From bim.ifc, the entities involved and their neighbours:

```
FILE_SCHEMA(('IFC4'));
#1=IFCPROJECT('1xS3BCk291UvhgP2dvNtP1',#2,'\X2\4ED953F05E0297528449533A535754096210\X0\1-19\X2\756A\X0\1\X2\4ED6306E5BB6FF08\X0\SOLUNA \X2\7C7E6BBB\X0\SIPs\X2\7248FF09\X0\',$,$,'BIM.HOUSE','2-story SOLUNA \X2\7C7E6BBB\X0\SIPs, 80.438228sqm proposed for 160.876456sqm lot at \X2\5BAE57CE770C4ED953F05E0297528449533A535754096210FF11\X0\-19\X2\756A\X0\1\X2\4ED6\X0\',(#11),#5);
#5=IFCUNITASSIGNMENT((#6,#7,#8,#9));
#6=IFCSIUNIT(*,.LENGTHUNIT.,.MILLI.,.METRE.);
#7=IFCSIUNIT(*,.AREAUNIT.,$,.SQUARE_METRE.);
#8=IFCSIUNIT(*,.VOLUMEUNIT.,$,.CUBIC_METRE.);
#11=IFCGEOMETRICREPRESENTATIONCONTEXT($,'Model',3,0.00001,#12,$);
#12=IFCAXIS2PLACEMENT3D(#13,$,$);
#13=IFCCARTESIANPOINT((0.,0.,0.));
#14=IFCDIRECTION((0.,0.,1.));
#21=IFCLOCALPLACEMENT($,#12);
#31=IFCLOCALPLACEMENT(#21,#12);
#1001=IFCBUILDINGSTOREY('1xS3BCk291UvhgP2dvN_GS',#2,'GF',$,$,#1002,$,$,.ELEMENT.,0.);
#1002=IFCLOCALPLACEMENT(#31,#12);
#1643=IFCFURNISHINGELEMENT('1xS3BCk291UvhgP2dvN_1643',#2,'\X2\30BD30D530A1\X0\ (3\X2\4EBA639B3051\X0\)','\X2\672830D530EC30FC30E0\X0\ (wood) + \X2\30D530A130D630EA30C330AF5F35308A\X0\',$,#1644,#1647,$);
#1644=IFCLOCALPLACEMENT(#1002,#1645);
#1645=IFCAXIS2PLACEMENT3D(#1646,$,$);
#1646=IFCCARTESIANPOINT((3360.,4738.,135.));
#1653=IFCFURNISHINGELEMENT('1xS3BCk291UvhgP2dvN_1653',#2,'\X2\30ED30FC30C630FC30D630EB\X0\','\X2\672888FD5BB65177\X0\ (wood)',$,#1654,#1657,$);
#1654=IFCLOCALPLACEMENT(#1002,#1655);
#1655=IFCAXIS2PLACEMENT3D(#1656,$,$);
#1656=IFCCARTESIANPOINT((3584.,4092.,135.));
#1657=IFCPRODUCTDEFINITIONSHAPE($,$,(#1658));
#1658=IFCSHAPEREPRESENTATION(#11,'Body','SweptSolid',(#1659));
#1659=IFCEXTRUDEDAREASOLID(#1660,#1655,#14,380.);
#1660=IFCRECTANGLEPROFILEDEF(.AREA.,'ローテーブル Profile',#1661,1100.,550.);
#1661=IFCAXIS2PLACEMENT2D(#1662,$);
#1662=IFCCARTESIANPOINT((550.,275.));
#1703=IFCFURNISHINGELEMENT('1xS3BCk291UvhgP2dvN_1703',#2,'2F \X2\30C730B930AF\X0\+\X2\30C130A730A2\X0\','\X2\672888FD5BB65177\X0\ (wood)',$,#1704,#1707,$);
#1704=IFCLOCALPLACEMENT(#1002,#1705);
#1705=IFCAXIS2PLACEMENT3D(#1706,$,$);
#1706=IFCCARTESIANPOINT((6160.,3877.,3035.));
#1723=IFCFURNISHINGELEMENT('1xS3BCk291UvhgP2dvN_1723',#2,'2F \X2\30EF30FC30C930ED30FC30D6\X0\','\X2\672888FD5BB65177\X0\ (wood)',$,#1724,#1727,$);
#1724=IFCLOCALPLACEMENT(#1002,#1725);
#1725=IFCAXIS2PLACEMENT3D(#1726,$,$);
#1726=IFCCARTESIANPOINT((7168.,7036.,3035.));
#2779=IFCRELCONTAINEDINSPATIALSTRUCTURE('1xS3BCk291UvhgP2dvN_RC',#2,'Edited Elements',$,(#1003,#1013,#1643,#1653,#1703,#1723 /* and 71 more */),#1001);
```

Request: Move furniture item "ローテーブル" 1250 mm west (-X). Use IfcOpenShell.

```python
import ifcopenshell
import ifcopenshell.api.geometry
import ifcopenshell.util.placement
import ifcopenshell.util.unit

model = ifcopenshell.open("bim.ifc")
unit_scale = ifcopenshell.util.unit.calculate_unit_scale(model)

item = model.by_guid("1xS3BCk291UvhgP2dvN_1653")
matrix = ifcopenshell.util.placement.get_local_placement(item.ObjectPlacement)
matrix[0, 3] -= 1.25 / unit_scale
ifcopenshell.api.geometry.edit_object_placement(model, product=item, matrix=matrix, is_si=False)

print(ifcopenshell.util.placement.get_local_placement(item.ObjectPlacement).round(3) + 0.0)

model.write("bim_edited.ifc")
```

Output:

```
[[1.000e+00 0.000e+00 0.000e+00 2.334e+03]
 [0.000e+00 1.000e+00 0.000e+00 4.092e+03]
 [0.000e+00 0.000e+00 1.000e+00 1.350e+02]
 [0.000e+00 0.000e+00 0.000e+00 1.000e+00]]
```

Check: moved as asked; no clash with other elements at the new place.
